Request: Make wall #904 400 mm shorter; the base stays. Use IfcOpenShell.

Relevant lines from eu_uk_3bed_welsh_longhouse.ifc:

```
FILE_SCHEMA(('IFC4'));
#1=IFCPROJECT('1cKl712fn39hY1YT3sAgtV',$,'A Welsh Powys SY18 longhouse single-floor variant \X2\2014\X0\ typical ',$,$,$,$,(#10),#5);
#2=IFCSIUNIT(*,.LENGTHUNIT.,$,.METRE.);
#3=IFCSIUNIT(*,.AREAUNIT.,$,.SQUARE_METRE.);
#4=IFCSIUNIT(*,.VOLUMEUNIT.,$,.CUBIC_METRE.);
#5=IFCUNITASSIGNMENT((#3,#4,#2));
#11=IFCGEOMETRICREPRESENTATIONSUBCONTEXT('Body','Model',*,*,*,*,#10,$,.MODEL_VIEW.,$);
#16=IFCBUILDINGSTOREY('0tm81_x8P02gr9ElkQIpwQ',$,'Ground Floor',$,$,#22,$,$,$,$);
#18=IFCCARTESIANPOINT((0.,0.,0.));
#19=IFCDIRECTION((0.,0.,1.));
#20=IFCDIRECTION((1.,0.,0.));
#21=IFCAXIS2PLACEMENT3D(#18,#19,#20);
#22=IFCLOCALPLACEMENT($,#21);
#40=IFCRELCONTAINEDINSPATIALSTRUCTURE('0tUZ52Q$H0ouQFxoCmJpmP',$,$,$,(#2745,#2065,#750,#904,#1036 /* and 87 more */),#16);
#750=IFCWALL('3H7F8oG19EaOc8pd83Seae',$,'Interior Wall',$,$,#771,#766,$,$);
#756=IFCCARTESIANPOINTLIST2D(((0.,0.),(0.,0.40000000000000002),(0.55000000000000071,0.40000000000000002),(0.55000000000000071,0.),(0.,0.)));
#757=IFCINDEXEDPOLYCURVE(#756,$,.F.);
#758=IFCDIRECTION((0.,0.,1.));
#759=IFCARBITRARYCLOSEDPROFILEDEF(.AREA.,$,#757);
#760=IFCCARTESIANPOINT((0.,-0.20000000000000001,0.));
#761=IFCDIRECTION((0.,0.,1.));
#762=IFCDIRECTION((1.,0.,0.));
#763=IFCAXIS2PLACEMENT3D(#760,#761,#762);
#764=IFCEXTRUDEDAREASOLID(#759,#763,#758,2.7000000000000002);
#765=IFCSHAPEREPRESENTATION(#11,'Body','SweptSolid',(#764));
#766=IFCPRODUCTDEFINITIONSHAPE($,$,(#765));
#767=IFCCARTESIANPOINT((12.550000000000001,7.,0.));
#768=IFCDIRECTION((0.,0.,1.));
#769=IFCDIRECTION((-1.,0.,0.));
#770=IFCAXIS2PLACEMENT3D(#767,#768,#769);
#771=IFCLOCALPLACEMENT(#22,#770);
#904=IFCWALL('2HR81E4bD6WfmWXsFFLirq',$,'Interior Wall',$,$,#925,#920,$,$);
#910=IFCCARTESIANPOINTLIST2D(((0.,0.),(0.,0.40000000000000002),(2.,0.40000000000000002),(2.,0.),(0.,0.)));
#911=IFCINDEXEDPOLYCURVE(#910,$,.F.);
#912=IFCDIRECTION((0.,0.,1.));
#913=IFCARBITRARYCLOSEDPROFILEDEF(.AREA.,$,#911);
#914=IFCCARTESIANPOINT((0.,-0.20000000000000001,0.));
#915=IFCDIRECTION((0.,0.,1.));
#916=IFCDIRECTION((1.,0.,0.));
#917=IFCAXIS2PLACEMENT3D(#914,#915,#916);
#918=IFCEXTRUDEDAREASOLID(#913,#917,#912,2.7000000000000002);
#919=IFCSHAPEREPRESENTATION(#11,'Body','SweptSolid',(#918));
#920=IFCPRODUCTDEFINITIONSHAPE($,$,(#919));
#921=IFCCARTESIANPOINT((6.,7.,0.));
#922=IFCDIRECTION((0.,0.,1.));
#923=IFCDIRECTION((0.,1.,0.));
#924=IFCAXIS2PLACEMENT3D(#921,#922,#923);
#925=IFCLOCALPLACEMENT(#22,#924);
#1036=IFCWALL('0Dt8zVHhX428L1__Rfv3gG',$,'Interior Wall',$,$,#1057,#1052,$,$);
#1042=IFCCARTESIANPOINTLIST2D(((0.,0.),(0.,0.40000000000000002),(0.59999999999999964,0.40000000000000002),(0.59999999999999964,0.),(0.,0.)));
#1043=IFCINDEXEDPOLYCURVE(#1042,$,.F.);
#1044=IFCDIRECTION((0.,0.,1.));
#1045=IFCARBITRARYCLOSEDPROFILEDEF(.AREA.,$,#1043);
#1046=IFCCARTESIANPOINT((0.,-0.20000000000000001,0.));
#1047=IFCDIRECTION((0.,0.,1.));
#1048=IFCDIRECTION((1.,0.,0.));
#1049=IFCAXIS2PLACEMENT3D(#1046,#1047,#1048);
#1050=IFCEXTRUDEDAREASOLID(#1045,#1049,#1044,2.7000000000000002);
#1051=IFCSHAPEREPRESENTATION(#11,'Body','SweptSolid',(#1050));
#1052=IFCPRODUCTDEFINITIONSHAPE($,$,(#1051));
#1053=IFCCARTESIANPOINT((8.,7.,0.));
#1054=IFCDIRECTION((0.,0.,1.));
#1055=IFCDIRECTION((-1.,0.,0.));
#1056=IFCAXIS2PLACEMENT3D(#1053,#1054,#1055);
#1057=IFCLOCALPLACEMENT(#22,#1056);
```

```python
import ifcopenshell
import ifcopenshell.geom
import ifcopenshell.util.representation
import ifcopenshell.util.shape
import ifcopenshell.util.unit

model = ifcopenshell.open("eu_uk_3bed_welsh_longhouse.ifc")
unit_scale = ifcopenshell.util.unit.calculate_unit_scale(model)
settings = ifcopenshell.geom.settings()


def volume(element):
    """Net volume in cubic metres, openings subtracted."""
    shape = ifcopenshell.geom.create_shape(settings, element)
    return ifcopenshell.util.shape.get_volume(shape.geometry)


wall = model.by_guid("2HR81E4bD6WfmWXsFFLirq")
before = volume(wall)

body = ifcopenshell.util.representation.get_representation(wall, "Model", "Body")
solid = body.Items[0]
old_height = solid.Depth
solid.Depth -= 0.4 / unit_scale
after = volume(wall)

print(f"height {old_height:g} -> {solid.Depth:g}, volume {before:.3f} -> {after:.3f} m3")

model.write("eu_uk_3bed_welsh_longhouse_edited.ifc")
```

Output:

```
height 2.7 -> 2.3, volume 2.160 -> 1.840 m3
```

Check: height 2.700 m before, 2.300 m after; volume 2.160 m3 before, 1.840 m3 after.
